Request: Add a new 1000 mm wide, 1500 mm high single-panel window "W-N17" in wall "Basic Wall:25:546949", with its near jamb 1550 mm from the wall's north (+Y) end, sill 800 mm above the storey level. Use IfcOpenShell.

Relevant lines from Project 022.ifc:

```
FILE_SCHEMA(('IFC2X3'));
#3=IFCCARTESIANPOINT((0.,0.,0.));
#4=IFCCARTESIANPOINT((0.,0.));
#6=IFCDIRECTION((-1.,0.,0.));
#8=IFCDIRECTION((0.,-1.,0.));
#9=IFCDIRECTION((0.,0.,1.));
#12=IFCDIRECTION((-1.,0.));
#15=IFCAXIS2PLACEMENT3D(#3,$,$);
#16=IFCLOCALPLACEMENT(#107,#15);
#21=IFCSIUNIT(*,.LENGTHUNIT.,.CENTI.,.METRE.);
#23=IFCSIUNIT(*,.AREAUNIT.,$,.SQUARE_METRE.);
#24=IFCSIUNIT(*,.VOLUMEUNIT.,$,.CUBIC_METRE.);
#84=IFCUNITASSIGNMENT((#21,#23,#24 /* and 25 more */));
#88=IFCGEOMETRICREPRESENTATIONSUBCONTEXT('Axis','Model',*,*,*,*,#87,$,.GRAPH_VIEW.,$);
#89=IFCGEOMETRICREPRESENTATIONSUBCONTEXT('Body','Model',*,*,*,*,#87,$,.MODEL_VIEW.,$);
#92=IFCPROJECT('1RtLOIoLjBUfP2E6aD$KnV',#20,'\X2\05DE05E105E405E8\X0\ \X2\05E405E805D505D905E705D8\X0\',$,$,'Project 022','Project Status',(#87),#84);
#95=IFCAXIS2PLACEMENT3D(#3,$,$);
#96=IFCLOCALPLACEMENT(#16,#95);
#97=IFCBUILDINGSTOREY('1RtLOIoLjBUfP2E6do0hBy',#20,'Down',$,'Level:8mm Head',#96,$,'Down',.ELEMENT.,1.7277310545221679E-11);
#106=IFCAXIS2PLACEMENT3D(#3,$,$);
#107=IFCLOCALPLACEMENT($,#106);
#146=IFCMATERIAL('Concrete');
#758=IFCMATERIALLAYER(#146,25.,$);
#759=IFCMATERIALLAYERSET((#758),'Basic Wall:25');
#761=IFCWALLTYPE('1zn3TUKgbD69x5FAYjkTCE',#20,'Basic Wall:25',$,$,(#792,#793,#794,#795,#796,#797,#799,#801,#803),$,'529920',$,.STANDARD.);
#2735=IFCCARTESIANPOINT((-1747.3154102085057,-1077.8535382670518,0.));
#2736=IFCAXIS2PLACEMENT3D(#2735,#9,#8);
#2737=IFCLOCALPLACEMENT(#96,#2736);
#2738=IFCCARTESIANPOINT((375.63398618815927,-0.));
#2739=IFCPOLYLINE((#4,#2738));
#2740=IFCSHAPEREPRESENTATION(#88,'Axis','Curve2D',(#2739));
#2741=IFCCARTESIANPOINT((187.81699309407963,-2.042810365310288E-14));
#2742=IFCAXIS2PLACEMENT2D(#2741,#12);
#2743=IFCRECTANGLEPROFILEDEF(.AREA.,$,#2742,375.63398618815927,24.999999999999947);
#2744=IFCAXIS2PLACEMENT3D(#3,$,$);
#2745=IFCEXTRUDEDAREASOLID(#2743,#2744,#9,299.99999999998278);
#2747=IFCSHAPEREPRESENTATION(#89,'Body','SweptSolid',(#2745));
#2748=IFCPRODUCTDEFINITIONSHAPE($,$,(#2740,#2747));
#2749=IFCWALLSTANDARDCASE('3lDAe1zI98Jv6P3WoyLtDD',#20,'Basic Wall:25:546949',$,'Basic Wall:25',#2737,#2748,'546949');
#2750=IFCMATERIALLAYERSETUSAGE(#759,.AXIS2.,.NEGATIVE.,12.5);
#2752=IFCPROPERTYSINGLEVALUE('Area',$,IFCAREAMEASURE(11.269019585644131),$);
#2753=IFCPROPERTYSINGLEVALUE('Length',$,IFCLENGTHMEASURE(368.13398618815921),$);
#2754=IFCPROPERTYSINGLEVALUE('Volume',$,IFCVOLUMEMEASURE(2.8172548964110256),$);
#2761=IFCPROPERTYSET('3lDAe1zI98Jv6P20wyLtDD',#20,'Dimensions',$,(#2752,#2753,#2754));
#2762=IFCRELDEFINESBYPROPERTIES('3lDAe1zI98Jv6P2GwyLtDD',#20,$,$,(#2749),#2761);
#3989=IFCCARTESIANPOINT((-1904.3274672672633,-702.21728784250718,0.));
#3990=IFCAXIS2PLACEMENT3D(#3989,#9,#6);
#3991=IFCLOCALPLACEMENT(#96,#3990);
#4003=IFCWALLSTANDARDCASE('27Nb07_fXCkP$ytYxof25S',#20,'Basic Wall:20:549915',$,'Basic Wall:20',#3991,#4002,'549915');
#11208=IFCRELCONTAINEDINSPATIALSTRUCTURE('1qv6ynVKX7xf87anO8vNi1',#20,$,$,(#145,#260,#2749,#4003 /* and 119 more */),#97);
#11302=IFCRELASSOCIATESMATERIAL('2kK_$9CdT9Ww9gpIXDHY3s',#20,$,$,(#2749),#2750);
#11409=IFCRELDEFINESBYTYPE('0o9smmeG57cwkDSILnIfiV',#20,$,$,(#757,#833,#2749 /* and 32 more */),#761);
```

```python
import numpy as np
import ifcopenshell
import ifcopenshell.api.feature
import ifcopenshell.api.geometry
import ifcopenshell.api.pset
import ifcopenshell.api.root
import ifcopenshell.api.spatial
import ifcopenshell.api.type
import ifcopenshell.geom
import ifcopenshell.util.element
import ifcopenshell.util.placement
import ifcopenshell.util.representation
import ifcopenshell.util.shape
import ifcopenshell.util.unit

model = ifcopenshell.open("Project 022.ifc")
unit_scale = ifcopenshell.util.unit.calculate_unit_scale(model)
area_scale = ifcopenshell.util.unit.calculate_unit_scale(model, "AREAUNIT")
volume_scale = ifcopenshell.util.unit.calculate_unit_scale(model, "VOLUMEUNIT")
settings = ifcopenshell.geom.settings()


def volume(element):
    """Net volume in cubic metres, openings subtracted."""
    shape = ifcopenshell.geom.create_shape(settings, element)
    return ifcopenshell.util.shape.get_volume(shape.geometry)


wall = model.by_id(2749)
storey = ifcopenshell.util.element.get_container(wall, ifc_class="IfcBuildingStorey")
context = ifcopenshell.util.representation.get_context(model, "Model", "Body", "MODEL_VIEW")
before = volume(wall)

width, height, from_end, sill = 1, 1.5, 1.55, 0.8  # metres

# The wall runs along its own X axis, and the end named is its -X end.
wall_shape = ifcopenshell.geom.create_shape(settings, wall)
x, y, z = ifcopenshell.util.shape.get_vertices(wall_shape.geometry).T
start = x.min() + from_end
face, thickness = float(y.min()), float(y.max() - y.min())
wall_matrix = ifcopenshell.util.placement.get_local_placement(wall.ObjectPlacement)
level = ifcopenshell.util.placement.get_local_placement(storey.ObjectPlacement)[2, 3]


def in_wall(x, y):
    """Placement at x, y metres in the wall's axes, at sill height."""
    matrix = wall_matrix.copy()
    matrix[:, 3] = wall_matrix @ np.array([x / unit_scale, y / unit_scale, 0.0, 1.0])
    matrix[2, 3] = level + sill / unit_scale
    return matrix


# Opening: a box that overshoots both wall faces by 50 mm.
opening = ifcopenshell.api.root.create_entity(model, ifc_class="IfcOpeningElement")
box = ifcopenshell.api.geometry.add_wall_representation(
    model, context=context, length=width, height=height, thickness=thickness + 0.1
)
ifcopenshell.api.geometry.assign_representation(model, product=opening, representation=box)
ifcopenshell.api.geometry.edit_object_placement(model, product=opening, matrix=in_wall(start, face - 0.05), is_si=False)
ifcopenshell.api.feature.add_feature(model, feature=opening, element=wall)

window = ifcopenshell.api.root.create_entity(model, ifc_class="IfcWindow", name="W-N17")
window.OverallWidth, window.OverallHeight = width / unit_scale, height / unit_scale
body = ifcopenshell.api.geometry.add_window_representation(
    model,
    context=context,
    overall_width=window.OverallWidth,
    overall_height=window.OverallHeight,
    partition_type="SINGLE_PANEL",
)
ifcopenshell.api.geometry.assign_representation(model, product=window, representation=body)
ifcopenshell.api.spatial.assign_container(model, products=[window], relating_structure=storey)
fills = ifcopenshell.api.feature.add_filling(model, opening=opening, element=window)
fills.OwnerHistory = window.OwnerHistory  # required in IFC2X3

# IFC2X3 keeps the operation on the window style.
style = ifcopenshell.api.root.create_entity(model, ifc_class="IfcWindowStyle", name="W-N17")
style.OperationType, style.ConstructionType = "SINGLE_PANEL", "NOTDEFINED"
style.ParameterTakesPrecedence = style.Sizeable = False
ifcopenshell.api.type.assign_type(model, related_objects=[window], relating_type=style)

# Centre the window in the wall's thickness.
ifcopenshell.api.geometry.edit_object_placement(model, product=window, matrix=in_wall(start, face), is_si=False)
window_shape = ifcopenshell.geom.create_shape(settings, window)
depth = ifcopenshell.util.shape.get_vertices(window_shape.geometry)[:, 1]
offset = face + thickness / 2 - (depth.min() + depth.max()) / 2
ifcopenshell.api.geometry.edit_object_placement(model, product=window, matrix=in_wall(start, offset), is_si=False)

after = volume(wall)

# Update the wall's stored quantities.
pset = model.by_id(ifcopenshell.util.element.get_pset(wall, "Dimensions", should_inherit=False)["id"])
ifcopenshell.api.pset.edit_pset(model, pset=pset, properties={
    "Area": model.create_entity("IfcAreaMeasure", after / thickness / area_scale),
    "Volume": model.create_entity("IfcVolumeMeasure", after / volume_scale),
})

print(f"wall volume {before:.3f} -> {after:.3f} m3")

model.write("Project 022_v2.ifc")
```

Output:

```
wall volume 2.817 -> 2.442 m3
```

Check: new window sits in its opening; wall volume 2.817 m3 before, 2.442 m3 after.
